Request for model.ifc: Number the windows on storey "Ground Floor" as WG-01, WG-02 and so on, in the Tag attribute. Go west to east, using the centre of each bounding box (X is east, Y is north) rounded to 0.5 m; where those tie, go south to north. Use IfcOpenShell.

First a look at what the model holds.

```python
import ifcopenshell
import ifcopenshell.util.element
import ifcopenshell.util.placement

model = ifcopenshell.open("model.ifc")
print(model.schema)
storey = next(s for s in model.by_type("IfcBuildingStorey") if s.Name == "Ground Floor")
windows = [e for e in ifcopenshell.util.element.get_decomposition(storey) if e.is_a("IfcWindow")]
for e in sorted(windows, key=lambda e: e.id()):
    origin = ifcopenshell.util.placement.get_local_placement(e.ObjectPlacement)[:3, 3]
    print(e.id(), e.Tag, e.Name, origin.round(2) + 0.0, sep=" | ")
```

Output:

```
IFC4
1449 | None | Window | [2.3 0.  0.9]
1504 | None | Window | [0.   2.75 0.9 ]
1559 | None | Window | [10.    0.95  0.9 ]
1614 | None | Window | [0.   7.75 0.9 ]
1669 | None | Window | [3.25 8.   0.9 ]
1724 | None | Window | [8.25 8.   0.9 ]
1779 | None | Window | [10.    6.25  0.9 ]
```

```python
import ifcopenshell
import ifcopenshell.geom
import ifcopenshell.util.element
import ifcopenshell.util.shape

model = ifcopenshell.open("model.ifc")
settings = ifcopenshell.geom.settings()
settings.set("use-world-coords", True)


def centre(element):
    shape = ifcopenshell.geom.create_shape(settings, element)
    return ifcopenshell.util.shape.get_bbox_centroid(shape.geometry)


storey = next(s for s in model.by_type("IfcBuildingStorey") if s.Name == "Ground Floor")
windows = [e for e in ifcopenshell.util.element.get_decomposition(storey) if e.is_a("IfcWindow")]

# Insertion points can sit at a corner or the storey origin, so sort by the geometry (in metres).
centres = {e: centre(e) for e in windows}
windows.sort(key=lambda e: (round(centres[e][0] / 0.5), centres[e][1]))

for i, e in enumerate(windows, start=1):
    number = f"WG-{i:02d}"
    e.Tag = number
    print(e.id(), number)

model.write("model_rev.ifc")
```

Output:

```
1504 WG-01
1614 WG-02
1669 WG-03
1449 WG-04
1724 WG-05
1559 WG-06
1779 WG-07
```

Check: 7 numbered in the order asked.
